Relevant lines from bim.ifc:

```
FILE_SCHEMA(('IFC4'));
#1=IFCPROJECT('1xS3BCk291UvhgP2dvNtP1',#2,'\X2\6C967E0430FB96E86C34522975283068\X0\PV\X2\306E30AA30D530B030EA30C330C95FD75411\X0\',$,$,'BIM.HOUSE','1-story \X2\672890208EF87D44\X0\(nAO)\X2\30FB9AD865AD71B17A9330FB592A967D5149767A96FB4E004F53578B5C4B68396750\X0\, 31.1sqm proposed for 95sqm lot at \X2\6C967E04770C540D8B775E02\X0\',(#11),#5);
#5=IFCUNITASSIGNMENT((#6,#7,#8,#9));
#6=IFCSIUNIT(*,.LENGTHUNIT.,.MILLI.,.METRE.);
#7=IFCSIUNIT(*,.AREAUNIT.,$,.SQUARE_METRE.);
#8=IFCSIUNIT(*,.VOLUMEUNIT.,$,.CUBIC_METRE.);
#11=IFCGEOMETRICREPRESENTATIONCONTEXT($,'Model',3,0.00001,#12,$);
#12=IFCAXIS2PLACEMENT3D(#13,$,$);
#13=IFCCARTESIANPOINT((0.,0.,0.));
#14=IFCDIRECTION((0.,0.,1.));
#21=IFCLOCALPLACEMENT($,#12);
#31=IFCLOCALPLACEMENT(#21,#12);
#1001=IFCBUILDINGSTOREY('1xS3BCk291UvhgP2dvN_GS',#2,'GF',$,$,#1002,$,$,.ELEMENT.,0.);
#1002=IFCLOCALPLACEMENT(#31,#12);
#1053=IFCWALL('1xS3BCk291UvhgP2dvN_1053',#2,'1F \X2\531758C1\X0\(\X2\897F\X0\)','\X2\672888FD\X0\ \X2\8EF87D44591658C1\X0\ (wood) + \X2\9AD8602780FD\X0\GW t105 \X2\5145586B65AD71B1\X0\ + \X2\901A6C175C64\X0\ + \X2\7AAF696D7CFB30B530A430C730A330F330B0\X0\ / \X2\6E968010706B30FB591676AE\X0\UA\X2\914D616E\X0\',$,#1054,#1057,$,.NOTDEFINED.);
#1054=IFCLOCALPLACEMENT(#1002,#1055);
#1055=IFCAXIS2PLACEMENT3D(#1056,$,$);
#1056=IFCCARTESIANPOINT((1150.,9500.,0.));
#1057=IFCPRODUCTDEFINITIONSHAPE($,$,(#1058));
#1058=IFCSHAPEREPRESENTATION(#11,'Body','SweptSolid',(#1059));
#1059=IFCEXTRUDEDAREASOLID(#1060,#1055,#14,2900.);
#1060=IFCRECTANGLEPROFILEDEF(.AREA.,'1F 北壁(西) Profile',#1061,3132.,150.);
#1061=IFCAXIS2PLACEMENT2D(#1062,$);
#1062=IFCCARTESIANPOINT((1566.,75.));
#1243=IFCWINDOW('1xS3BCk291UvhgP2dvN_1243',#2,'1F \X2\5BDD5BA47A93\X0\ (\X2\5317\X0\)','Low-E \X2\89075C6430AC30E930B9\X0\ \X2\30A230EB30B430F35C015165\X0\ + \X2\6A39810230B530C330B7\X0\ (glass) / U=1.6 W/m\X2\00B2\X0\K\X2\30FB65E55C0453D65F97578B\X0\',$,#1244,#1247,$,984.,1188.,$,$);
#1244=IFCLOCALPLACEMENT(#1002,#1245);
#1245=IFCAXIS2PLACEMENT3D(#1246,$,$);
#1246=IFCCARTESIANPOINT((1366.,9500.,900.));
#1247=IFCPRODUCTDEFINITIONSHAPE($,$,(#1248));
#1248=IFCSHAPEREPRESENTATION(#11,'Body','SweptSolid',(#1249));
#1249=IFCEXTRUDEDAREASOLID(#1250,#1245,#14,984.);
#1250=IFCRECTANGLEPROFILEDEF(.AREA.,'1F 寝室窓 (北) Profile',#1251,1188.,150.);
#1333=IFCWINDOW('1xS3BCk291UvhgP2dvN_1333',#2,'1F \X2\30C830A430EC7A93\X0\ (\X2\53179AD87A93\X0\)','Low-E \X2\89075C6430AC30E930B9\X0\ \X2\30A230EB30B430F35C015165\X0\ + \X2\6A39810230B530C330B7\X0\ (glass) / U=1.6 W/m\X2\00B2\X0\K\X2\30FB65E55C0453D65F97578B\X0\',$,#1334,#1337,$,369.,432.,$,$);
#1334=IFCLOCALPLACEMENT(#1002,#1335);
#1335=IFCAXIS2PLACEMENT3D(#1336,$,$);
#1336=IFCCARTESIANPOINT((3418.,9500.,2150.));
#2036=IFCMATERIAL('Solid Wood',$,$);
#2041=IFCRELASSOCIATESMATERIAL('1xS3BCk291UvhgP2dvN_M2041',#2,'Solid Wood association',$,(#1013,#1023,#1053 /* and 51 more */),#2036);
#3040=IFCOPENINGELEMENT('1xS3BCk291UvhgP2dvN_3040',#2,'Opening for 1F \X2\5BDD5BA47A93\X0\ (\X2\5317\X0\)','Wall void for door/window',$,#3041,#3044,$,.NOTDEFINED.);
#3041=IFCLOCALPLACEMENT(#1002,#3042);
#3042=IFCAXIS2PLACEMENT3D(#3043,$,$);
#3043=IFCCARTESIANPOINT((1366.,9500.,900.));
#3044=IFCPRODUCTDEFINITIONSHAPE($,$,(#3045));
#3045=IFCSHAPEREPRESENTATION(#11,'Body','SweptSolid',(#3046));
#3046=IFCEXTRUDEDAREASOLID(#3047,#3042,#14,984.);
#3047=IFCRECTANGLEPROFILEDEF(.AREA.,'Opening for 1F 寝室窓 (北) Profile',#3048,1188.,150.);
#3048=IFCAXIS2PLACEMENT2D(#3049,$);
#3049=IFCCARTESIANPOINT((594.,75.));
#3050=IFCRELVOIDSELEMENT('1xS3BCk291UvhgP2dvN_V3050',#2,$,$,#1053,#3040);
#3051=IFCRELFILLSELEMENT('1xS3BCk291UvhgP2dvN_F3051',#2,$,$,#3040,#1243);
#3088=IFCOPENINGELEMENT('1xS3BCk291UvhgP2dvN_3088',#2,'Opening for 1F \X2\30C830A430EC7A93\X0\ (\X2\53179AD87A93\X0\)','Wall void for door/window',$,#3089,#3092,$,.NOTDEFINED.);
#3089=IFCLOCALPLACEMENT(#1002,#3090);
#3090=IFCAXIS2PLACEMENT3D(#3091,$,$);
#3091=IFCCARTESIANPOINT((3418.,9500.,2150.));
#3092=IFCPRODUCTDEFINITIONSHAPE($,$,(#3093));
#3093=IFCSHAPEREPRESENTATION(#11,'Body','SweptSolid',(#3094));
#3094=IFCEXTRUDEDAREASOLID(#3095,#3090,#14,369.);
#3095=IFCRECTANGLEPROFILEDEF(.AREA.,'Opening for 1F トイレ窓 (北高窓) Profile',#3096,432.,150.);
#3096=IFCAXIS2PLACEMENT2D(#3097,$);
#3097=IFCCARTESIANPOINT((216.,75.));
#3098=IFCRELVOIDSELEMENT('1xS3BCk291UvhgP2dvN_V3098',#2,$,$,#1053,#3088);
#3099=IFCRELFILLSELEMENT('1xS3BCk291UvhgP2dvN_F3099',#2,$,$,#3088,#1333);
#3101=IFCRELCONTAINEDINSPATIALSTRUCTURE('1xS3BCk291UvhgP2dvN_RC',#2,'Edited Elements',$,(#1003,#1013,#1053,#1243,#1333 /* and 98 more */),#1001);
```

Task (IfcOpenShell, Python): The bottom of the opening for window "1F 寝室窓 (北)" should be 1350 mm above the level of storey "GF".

```python
import numpy as np
import ifcopenshell
import ifcopenshell.api.geometry
import ifcopenshell.geom
import ifcopenshell.util.element
import ifcopenshell.util.placement
import ifcopenshell.util.shape
import ifcopenshell.util.unit

model = ifcopenshell.open("bim.ifc")
unit_scale = ifcopenshell.util.unit.calculate_unit_scale(model)

window = model.by_id(1243)
opening = window.FillsVoids[0].RelatingOpeningElement
storey = ifcopenshell.util.element.get_container(window, ifc_class="IfcBuildingStorey")
level = ifcopenshell.util.placement.get_local_placement(storey.ObjectPlacement)[2, 3]

# The opening's origin need not be at the sill, so measure its lowest point.
shape = ifcopenshell.geom.create_shape(ifcopenshell.geom.settings(), opening)
bottom = ifcopenshell.util.shape.get_shape_bottom_elevation(shape, shape.geometry) / unit_scale
dz = level + 1350.0 - bottom

shift = np.array([0.0, 0.0, dz])
# The window is not placed relative to its opening, so move both.
for product in (opening, window):
    matrix = ifcopenshell.util.placement.get_local_placement(product.ObjectPlacement)
    matrix[:3, 3] += shift
    ifcopenshell.api.geometry.edit_object_placement(model, product=product, matrix=matrix, is_si=False)

print(f"moved by {dz * unit_scale:+.3f} m")

model.write("bim_updated.ifc")
```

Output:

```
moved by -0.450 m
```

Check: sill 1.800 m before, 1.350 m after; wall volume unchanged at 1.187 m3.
